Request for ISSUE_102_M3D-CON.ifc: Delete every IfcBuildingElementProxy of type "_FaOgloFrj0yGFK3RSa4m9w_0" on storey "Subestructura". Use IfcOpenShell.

First a look at what the model holds.

```python
import ifcopenshell
import ifcopenshell.util.element

model = ifcopenshell.open("ISSUE_102_M3D-CON.ifc")
print(model.schema)
storey = next(s for s in model.by_type("IfcBuildingStorey") if s.Name == "Subestructura")
proxies = [e for e in ifcopenshell.util.element.get_decomposition(storey) if e.is_a("IfcBuildingElementProxy")]
seen = {}
for e in proxies:
    element_type = ifcopenshell.util.element.get_type(e)
    name = element_type.Name if element_type not in (None, e) else None
    seen[name] = seen.get(name, 0) + 1
for name, count in sorted(seen.items(), key=str):
    print(count, "x", name)
```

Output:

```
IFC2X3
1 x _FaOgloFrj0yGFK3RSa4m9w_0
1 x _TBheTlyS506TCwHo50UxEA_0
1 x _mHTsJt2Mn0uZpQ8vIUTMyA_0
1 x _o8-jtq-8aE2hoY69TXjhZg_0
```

```python
import ifcopenshell
import ifcopenshell.api.root
import ifcopenshell.util.element

model = ifcopenshell.open("ISSUE_102_M3D-CON.ifc")

storey = next(s for s in model.by_type("IfcBuildingStorey") if s.Name == "Subestructura")
proxies = [e for e in ifcopenshell.util.element.get_decomposition(storey) if e.is_a("IfcBuildingElementProxy")]
targets = [e for e in proxies if (t := ifcopenshell.util.element.get_type(e)) not in (None, e) and t.Name == "_FaOgloFrj0yGFK3RSa4m9w_0"]

for e in targets:
    ifcopenshell.api.root.remove_product(model, product=e)
print(len(targets), "removed")

model.write("ISSUE_102_M3D-CON_v2.ifc")
```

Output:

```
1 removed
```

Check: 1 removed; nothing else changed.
